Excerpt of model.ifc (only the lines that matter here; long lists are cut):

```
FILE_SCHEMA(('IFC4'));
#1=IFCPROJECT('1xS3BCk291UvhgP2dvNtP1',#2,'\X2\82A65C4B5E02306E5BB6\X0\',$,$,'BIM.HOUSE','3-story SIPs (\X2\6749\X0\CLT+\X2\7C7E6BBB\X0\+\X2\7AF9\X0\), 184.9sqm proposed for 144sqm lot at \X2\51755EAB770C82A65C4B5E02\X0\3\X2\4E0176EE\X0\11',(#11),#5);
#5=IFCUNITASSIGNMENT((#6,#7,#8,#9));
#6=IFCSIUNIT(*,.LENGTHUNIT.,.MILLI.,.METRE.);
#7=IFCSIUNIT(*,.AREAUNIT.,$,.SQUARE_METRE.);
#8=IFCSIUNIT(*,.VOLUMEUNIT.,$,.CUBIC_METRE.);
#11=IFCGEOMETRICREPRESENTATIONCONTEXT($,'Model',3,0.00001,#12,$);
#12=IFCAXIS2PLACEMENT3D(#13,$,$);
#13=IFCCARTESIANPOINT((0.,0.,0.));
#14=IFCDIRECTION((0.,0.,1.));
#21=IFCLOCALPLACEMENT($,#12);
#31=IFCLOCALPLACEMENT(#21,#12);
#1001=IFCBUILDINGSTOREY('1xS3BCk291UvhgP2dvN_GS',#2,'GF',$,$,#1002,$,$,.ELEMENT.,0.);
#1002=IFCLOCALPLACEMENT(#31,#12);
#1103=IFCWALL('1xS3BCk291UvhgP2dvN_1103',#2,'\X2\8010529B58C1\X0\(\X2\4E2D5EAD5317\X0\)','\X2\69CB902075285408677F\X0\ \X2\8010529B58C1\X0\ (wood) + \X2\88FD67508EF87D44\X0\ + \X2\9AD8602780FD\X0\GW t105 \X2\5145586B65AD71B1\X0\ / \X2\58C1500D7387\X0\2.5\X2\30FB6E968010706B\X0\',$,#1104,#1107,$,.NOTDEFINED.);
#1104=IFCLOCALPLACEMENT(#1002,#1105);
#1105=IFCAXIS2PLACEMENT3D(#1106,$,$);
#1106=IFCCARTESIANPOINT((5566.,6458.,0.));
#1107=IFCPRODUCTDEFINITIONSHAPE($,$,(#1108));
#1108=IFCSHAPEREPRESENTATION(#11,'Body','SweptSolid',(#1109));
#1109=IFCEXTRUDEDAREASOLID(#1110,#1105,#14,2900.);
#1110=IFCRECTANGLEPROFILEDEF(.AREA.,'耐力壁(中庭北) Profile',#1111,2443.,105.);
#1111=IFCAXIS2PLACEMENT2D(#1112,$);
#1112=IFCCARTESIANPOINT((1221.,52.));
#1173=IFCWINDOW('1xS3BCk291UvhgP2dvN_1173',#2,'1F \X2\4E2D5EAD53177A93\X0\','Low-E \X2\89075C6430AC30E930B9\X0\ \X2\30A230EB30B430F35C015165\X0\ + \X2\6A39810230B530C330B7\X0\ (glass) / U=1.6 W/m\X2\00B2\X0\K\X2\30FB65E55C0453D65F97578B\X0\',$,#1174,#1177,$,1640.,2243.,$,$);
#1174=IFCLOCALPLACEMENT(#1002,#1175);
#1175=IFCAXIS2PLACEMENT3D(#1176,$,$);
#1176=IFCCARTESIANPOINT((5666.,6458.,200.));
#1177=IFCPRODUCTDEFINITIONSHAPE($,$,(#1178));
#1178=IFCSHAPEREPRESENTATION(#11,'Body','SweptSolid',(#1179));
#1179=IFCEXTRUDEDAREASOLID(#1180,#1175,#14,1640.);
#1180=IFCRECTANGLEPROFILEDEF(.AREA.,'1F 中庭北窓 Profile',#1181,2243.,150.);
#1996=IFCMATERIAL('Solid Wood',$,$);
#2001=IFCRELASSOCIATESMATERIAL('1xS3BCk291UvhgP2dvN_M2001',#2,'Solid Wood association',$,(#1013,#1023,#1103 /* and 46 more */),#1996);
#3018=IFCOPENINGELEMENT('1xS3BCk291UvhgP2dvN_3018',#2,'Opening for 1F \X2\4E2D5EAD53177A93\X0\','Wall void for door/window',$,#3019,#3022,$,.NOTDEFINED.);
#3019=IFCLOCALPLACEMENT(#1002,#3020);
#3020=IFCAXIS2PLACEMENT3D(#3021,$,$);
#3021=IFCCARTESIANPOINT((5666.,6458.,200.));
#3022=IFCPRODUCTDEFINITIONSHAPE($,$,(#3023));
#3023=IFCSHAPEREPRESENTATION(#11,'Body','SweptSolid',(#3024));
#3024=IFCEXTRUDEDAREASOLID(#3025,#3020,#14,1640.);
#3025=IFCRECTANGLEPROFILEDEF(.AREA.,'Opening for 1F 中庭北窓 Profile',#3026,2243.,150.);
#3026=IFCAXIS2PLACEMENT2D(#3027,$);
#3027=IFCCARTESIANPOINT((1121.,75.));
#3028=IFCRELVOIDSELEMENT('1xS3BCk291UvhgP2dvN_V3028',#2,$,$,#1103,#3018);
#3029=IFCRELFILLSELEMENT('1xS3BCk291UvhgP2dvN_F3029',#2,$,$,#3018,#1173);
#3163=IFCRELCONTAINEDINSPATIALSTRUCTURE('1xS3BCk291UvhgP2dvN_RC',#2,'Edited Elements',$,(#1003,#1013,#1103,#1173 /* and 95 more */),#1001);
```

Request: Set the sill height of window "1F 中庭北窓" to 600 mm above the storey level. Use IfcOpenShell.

```python
import numpy as np
import ifcopenshell
import ifcopenshell.api.geometry
import ifcopenshell.geom
import ifcopenshell.util.element
import ifcopenshell.util.placement
import ifcopenshell.util.shape
import ifcopenshell.util.unit

model = ifcopenshell.open("model.ifc")
unit_scale = ifcopenshell.util.unit.calculate_unit_scale(model)

window = model.by_guid("1xS3BCk291UvhgP2dvN_1173")
opening = window.FillsVoids[0].RelatingOpeningElement
storey = ifcopenshell.util.element.get_container(window, ifc_class="IfcBuildingStorey")
level = ifcopenshell.util.placement.get_local_placement(storey.ObjectPlacement)[2, 3]

# The opening's origin need not be at the sill, so measure its lowest point.
shape = ifcopenshell.geom.create_shape(ifcopenshell.geom.settings(), opening)
bottom = ifcopenshell.util.shape.get_shape_bottom_elevation(shape, shape.geometry) / unit_scale
dz = level + 600.0 - bottom

shift = np.array([0.0, 0.0, dz])
# The window is not placed relative to its opening, so move both.
for product in (opening, window):
    matrix = ifcopenshell.util.placement.get_local_placement(product.ObjectPlacement)
    matrix[:3, 3] += shift
    ifcopenshell.api.geometry.edit_object_placement(model, product=product, matrix=matrix, is_si=False)

print(f"moved by {dz * unit_scale:+.3f} m")

model.write("model_v2.ifc")
```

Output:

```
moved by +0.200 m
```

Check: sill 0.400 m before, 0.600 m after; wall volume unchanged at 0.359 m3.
